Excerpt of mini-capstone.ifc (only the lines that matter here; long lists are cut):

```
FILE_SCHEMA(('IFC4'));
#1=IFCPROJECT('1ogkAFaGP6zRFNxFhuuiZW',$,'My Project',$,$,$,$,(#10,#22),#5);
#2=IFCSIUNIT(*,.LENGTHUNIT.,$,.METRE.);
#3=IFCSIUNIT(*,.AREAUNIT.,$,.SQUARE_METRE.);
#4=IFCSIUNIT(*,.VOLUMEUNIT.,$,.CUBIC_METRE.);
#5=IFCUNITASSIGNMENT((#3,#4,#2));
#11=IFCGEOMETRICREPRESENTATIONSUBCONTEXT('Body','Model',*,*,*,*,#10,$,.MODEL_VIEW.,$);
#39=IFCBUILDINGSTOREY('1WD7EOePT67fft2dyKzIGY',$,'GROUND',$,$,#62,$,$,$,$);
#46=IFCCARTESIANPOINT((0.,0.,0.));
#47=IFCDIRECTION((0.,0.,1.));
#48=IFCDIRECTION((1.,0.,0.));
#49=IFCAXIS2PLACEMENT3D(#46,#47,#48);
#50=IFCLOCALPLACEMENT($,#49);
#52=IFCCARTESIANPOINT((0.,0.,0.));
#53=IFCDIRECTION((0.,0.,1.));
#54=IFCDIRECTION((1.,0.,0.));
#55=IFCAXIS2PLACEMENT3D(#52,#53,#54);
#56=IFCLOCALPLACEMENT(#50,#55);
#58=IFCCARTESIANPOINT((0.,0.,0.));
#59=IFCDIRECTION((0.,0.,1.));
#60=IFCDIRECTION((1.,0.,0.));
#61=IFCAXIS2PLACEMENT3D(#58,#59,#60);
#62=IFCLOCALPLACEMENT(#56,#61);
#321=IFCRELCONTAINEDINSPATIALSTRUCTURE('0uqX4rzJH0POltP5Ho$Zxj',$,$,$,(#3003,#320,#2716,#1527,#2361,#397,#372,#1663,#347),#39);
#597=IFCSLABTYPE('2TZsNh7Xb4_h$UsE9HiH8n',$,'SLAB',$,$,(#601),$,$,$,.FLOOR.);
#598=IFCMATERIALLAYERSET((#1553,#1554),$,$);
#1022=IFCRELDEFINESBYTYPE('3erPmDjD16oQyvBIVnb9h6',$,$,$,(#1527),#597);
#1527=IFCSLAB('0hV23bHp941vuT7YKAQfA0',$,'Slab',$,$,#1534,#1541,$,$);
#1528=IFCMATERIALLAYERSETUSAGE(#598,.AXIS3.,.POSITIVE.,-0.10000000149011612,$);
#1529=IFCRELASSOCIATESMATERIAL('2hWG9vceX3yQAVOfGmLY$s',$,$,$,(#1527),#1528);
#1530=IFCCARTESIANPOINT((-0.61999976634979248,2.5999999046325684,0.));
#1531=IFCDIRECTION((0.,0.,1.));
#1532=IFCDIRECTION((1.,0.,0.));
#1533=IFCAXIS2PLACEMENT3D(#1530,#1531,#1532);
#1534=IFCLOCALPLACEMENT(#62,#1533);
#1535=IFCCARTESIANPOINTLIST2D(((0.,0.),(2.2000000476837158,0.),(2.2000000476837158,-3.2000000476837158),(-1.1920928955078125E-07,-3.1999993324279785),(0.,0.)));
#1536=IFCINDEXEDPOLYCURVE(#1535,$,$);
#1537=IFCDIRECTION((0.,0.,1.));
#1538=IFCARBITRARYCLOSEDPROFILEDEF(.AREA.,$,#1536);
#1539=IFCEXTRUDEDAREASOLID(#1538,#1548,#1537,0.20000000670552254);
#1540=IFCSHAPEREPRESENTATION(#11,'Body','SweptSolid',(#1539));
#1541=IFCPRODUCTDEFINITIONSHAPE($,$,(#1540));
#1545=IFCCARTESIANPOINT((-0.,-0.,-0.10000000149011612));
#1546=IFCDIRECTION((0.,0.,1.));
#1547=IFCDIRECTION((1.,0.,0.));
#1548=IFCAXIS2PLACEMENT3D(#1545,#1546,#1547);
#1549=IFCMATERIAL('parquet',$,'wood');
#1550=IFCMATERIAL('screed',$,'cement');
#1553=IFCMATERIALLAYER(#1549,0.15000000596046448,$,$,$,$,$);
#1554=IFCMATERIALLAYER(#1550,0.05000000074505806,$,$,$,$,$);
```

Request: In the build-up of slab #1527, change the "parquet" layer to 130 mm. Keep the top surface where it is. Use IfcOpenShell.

```python
import ifcopenshell
import ifcopenshell.util.element
import ifcopenshell.util.representation
import ifcopenshell.util.unit

model = ifcopenshell.open("mini-capstone.ifc")
unit_scale = ifcopenshell.util.unit.calculate_unit_scale(model)

layer_set = model.by_id(598)
layer = next(l for l in layer_set.MaterialLayers if l.Material and l.Material.Name == "parquet")
change = 0.13 / unit_scale - layer.LayerThickness
layer.LayerThickness += change

# Geometry does not follow the layer set by itself.
slabs = [e for e in ifcopenshell.util.element.get_elements_by_material(model, layer_set) if e.is_a("IfcSlab")]
for slab in sorted(slabs, key=lambda e: e.id()):
    body = ifcopenshell.util.representation.get_representation(slab, "Model", "Body")
    solid = body.Items[0]
    old_depth = solid.Depth
    solid.Depth += change
    # Extruded upwards: lower the start of the extrusion so the top stays.
    x, y, z = solid.Position.Location.Coordinates
    solid.Position.Location = model.createIfcCartesianPoint((x, y, z - change))
    print(slab.id(), f"{old_depth:g} -> {solid.Depth:g}")

# The layers are counted up from the underside, which has moved.
for usage in {ifcopenshell.util.element.get_material(slab) for slab in slabs}:
    usage.OffsetFromReferenceLine -= change

model.write("mini-capstone-out.ifc")
```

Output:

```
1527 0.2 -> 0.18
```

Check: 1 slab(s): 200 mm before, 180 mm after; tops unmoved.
